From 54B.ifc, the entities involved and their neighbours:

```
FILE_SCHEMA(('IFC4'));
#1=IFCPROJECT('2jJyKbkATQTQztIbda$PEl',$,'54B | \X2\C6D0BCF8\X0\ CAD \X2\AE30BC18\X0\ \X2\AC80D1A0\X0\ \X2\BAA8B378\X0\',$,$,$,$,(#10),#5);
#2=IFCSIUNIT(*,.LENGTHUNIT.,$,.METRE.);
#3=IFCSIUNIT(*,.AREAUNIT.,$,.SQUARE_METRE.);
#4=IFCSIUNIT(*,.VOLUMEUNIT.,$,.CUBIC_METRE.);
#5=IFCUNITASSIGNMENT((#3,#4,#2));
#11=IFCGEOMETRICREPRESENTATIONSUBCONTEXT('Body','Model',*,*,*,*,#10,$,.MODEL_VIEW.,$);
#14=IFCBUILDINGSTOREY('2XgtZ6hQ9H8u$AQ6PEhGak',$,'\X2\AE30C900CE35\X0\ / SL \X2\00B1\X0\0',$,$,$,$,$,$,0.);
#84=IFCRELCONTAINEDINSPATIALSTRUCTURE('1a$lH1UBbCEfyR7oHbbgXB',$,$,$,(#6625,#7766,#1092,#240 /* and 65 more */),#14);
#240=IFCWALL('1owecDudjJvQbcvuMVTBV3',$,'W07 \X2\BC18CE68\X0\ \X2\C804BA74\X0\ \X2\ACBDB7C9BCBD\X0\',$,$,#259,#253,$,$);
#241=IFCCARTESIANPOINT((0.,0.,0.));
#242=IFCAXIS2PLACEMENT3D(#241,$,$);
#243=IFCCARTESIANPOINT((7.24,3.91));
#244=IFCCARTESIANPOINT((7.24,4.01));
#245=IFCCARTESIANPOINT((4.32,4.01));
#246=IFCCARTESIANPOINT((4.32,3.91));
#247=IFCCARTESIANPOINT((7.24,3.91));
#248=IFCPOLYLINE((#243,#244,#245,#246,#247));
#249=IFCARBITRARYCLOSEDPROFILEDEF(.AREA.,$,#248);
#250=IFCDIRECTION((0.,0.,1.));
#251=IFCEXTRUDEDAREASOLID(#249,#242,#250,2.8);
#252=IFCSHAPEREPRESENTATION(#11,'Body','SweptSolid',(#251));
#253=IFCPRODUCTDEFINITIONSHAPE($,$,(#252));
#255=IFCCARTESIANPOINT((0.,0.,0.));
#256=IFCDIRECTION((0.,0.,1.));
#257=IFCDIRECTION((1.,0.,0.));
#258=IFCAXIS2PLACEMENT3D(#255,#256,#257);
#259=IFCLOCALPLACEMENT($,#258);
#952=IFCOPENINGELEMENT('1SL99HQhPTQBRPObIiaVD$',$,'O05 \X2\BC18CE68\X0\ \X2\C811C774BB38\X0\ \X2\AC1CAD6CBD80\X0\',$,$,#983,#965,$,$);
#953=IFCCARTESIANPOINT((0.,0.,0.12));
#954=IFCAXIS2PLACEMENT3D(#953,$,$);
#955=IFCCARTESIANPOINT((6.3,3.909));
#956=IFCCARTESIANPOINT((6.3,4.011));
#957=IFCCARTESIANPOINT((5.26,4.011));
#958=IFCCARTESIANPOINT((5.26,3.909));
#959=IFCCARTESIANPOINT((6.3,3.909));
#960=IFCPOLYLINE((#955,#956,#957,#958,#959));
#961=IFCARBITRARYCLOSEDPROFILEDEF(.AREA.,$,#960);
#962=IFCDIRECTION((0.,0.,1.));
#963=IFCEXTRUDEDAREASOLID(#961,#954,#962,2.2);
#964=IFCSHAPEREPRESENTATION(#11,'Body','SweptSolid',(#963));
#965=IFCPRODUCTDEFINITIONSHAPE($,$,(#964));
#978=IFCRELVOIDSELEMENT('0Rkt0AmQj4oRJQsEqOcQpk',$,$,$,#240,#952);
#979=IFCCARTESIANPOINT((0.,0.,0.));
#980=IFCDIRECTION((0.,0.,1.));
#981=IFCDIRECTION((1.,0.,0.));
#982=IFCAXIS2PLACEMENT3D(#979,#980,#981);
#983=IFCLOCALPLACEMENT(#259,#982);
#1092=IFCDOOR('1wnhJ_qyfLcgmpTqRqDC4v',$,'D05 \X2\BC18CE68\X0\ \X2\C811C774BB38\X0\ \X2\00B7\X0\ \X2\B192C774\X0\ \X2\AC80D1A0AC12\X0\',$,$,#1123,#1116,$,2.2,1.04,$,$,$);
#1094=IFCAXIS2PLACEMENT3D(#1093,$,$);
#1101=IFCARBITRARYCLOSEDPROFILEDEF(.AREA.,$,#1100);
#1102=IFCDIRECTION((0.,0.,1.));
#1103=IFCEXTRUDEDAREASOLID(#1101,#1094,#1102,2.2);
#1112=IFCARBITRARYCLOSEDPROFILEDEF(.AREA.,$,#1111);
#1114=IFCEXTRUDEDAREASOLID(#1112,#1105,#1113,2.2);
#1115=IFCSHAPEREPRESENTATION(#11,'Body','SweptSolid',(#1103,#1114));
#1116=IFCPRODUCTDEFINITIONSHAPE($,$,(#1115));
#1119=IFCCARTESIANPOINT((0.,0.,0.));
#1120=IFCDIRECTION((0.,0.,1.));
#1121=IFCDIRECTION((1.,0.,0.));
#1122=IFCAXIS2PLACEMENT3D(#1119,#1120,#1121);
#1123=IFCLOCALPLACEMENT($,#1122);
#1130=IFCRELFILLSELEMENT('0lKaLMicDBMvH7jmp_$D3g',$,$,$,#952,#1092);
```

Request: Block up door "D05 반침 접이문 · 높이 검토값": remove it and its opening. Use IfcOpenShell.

```python
import ifcopenshell
import ifcopenshell.api.feature
import ifcopenshell.api.root
import ifcopenshell.geom
import ifcopenshell.util.shape

model = ifcopenshell.open("54B.ifc")
settings = ifcopenshell.geom.settings()


def volume(element):
    """Net volume in cubic metres, openings subtracted."""
    shape = ifcopenshell.geom.create_shape(settings, element)
    return ifcopenshell.util.shape.get_volume(shape.geometry)


door = model.by_guid("1wnhJ_qyfLcgmpTqRqDC4v")
opening = door.FillsVoids[0].RelatingOpeningElement
wall = opening.VoidsElements[0].RelatingBuildingElement
before = volume(wall)

ifcopenshell.api.root.remove_product(model, product=door)
ifcopenshell.api.feature.remove_feature(model, feature=opening)

after = volume(wall)

print(f"wall volume {before:.3f} -> {after:.3f} m3")

model.write("54B_updated.ifc")
```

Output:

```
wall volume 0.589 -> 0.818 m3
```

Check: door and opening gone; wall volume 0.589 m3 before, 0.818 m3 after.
